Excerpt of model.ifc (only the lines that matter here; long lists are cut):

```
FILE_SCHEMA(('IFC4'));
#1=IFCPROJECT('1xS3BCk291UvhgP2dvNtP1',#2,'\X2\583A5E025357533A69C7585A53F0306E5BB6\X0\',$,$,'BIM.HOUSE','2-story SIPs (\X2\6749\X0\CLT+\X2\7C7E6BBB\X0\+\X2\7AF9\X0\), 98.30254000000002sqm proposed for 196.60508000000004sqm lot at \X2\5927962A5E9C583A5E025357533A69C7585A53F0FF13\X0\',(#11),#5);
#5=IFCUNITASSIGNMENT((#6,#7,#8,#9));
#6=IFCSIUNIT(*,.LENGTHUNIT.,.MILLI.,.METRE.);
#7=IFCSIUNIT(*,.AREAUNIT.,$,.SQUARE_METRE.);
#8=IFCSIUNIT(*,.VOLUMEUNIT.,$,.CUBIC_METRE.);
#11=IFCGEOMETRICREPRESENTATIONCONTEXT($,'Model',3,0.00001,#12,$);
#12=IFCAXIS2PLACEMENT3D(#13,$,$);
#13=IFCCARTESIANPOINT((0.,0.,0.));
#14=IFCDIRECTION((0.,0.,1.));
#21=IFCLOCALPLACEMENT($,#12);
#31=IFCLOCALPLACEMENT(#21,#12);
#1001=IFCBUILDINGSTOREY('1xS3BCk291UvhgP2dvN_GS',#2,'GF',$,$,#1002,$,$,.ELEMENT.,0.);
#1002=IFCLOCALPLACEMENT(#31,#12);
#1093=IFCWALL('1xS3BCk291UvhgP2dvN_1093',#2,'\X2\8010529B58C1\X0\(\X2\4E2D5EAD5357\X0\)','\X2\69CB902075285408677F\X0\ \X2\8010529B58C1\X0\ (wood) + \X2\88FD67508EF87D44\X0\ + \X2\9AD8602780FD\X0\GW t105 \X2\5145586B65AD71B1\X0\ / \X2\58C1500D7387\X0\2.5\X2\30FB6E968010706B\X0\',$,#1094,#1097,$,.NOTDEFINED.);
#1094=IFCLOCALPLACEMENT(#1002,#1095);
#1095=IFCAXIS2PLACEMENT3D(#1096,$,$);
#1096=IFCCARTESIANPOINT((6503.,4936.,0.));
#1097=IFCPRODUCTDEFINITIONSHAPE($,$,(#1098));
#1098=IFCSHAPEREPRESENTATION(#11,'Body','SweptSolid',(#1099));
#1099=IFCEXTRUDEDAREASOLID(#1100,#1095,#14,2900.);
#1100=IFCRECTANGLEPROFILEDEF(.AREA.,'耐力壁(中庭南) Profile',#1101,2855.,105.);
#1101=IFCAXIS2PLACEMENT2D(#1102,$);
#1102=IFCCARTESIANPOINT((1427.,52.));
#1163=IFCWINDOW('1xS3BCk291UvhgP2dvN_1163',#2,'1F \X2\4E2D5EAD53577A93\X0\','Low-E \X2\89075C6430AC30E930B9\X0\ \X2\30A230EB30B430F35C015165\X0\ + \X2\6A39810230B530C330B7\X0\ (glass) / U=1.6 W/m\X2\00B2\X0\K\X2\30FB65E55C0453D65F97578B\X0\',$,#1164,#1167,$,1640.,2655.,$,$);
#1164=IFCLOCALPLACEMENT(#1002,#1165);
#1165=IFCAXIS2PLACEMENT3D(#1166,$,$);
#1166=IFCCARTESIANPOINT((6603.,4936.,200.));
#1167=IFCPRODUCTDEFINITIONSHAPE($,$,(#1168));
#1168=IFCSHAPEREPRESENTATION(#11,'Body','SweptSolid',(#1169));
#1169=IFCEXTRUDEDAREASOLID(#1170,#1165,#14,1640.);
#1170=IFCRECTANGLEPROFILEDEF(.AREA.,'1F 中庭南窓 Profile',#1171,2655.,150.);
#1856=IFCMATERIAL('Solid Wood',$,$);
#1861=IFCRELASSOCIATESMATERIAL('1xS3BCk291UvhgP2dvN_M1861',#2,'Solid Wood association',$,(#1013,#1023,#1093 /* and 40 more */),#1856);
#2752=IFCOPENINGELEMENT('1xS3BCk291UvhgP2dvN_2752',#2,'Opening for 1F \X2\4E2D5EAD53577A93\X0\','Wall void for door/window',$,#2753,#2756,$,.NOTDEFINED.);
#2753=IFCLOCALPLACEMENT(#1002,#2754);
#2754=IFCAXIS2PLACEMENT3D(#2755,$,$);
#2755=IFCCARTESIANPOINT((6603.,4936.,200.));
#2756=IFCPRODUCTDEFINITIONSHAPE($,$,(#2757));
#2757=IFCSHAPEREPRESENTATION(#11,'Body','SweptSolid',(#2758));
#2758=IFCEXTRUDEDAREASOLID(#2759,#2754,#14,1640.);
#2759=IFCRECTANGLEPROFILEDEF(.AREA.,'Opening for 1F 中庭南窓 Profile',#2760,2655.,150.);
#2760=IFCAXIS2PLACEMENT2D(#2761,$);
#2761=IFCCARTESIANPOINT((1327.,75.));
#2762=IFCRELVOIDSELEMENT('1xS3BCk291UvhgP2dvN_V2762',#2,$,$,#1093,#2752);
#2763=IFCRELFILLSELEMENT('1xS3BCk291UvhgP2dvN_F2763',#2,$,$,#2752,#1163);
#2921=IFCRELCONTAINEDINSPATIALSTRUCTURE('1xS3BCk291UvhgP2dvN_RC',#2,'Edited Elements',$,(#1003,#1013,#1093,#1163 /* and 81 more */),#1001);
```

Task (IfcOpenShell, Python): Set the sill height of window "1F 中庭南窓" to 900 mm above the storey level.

```python
import numpy as np
import ifcopenshell
import ifcopenshell.api.geometry
import ifcopenshell.geom
import ifcopenshell.util.element
import ifcopenshell.util.placement
import ifcopenshell.util.shape
import ifcopenshell.util.unit

model = ifcopenshell.open("model.ifc")
unit_scale = ifcopenshell.util.unit.calculate_unit_scale(model)

window = model.by_guid("1xS3BCk291UvhgP2dvN_1163")
opening = window.FillsVoids[0].RelatingOpeningElement
storey = ifcopenshell.util.element.get_container(window, ifc_class="IfcBuildingStorey")
level = ifcopenshell.util.placement.get_local_placement(storey.ObjectPlacement)[2, 3]

# The opening's origin need not be at the sill, so measure its lowest point.
shape = ifcopenshell.geom.create_shape(ifcopenshell.geom.settings(), opening)
bottom = ifcopenshell.util.shape.get_shape_bottom_elevation(shape, shape.geometry) / unit_scale
dz = level + 0.9 / unit_scale - bottom

shift = np.array([0.0, 0.0, dz])
# The window is not placed relative to its opening, so move both.
for product in (opening, window):
    matrix = ifcopenshell.util.placement.get_local_placement(product.ObjectPlacement)
    matrix[:3, 3] += shift
    ifcopenshell.api.geometry.edit_object_placement(model, product=product, matrix=matrix, is_si=False)

print(f"moved by {dz * unit_scale:+.3f} m")

model.write("model_rev.ifc")
```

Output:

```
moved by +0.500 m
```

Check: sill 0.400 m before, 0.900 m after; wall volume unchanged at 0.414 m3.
